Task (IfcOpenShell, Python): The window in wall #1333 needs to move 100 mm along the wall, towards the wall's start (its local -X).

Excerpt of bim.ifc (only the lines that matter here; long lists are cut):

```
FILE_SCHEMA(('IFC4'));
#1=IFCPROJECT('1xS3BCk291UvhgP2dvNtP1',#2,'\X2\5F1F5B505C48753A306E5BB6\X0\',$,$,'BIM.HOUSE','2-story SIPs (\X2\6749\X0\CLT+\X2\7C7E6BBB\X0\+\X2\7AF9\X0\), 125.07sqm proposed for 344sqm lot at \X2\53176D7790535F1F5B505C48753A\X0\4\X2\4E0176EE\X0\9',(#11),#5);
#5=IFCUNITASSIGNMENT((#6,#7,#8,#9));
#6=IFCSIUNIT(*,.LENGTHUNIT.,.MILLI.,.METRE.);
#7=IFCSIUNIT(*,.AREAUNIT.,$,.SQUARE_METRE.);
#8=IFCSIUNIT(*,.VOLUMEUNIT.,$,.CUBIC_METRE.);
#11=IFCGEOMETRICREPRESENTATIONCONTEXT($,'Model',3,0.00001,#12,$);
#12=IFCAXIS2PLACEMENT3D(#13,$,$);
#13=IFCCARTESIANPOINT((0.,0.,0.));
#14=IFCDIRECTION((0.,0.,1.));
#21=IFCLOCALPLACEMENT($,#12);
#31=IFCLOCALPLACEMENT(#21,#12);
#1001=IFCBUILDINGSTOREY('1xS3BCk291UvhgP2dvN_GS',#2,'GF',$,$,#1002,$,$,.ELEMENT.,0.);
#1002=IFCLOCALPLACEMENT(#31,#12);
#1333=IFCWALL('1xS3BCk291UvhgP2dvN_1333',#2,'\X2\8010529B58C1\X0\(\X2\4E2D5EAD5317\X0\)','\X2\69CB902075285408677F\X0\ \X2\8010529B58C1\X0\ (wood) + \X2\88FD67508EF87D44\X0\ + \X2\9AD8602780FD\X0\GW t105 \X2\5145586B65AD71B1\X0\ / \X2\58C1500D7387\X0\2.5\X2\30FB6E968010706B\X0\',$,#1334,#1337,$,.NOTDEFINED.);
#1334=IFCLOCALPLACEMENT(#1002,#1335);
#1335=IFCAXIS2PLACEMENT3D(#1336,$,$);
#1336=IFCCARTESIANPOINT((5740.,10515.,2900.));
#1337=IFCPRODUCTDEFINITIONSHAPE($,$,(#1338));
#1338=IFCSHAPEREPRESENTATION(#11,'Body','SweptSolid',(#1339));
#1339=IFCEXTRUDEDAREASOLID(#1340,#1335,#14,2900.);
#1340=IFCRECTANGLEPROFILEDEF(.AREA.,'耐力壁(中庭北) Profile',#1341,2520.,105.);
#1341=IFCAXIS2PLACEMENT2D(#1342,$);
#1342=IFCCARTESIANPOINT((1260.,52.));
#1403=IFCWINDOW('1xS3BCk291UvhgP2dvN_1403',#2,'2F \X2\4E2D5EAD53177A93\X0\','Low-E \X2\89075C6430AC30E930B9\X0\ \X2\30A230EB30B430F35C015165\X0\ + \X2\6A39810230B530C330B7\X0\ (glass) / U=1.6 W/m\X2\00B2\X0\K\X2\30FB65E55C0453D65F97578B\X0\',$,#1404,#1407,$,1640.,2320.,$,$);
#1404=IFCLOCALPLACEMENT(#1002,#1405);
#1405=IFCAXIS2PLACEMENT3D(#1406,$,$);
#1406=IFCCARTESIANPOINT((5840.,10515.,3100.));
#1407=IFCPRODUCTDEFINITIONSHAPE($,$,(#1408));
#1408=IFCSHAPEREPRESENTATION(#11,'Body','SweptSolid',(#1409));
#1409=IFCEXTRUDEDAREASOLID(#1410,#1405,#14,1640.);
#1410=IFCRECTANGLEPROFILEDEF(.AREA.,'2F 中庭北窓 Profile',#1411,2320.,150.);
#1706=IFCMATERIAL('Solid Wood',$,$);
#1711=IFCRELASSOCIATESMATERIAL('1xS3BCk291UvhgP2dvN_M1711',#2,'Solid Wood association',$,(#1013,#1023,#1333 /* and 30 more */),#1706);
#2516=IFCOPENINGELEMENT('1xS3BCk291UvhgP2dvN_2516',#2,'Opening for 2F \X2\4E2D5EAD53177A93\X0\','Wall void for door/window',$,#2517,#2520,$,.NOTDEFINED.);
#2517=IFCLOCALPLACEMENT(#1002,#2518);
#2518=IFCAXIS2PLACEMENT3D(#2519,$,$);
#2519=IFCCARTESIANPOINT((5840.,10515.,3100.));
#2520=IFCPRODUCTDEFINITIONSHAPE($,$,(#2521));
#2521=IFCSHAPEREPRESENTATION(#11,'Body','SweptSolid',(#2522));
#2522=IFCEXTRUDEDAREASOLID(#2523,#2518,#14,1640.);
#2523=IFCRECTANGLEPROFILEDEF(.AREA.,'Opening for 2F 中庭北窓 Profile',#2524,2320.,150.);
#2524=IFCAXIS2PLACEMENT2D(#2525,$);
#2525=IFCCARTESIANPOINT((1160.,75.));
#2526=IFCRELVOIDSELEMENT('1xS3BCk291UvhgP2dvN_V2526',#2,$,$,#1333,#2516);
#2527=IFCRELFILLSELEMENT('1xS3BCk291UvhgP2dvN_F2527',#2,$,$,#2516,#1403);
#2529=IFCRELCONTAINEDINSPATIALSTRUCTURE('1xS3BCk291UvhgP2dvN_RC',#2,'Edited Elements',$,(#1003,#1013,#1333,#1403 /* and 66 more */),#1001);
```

```python
import ifcopenshell
import ifcopenshell.api.geometry
import ifcopenshell.util.placement

model = ifcopenshell.open("bim.ifc")

window = model.by_guid("1xS3BCk291UvhgP2dvN_1403")
opening = window.FillsVoids[0].RelatingOpeningElement
wall = opening.VoidsElements[0].RelatingBuildingElement

wall_matrix = ifcopenshell.util.placement.get_local_placement(wall.ObjectPlacement)
shift = wall_matrix[:3, 0] * -100.0
before = ifcopenshell.util.placement.get_local_placement(window.ObjectPlacement)[:3, 3].copy()

# The window is not placed relative to its opening, so move both.
for product in (opening, window):
    matrix = ifcopenshell.util.placement.get_local_placement(product.ObjectPlacement)
    matrix[:3, 3] += shift
    ifcopenshell.api.geometry.edit_object_placement(model, product=product, matrix=matrix, is_si=False)

after = ifcopenshell.util.placement.get_local_placement(window.ObjectPlacement)[:3, 3]
print("window moved by", (after - before).round(3) + 0.0)

model.write("bim_edited.ifc")
```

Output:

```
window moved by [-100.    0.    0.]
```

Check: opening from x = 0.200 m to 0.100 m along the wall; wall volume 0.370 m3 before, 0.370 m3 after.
